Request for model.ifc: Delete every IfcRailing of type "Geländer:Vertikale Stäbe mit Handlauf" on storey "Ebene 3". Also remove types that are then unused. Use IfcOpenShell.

First a look at what the model holds.

```python
import ifcopenshell
import ifcopenshell.util.element

model = ifcopenshell.open("model.ifc")
print(model.schema)
storey = next(s for s in model.by_type("IfcBuildingStorey") if s.Name == "Ebene 3")
railings = [e for e in ifcopenshell.util.element.get_decomposition(storey) if e.is_a("IfcRailing")]
seen = {}
for e in railings:
    element_type = ifcopenshell.util.element.get_type(e)
    name = element_type.Name if element_type not in (None, e) else None
    seen[name] = seen.get(name, 0) + 1
for name, count in sorted(seen.items(), key=str):
    print(count, "x", name)
```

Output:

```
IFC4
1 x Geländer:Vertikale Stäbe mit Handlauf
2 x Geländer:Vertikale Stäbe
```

```python
import ifcopenshell
import ifcopenshell.api.root
import ifcopenshell.util.element

model = ifcopenshell.open("model.ifc")

storey = next(s for s in model.by_type("IfcBuildingStorey") if s.Name == "Ebene 3")
railings = [e for e in ifcopenshell.util.element.get_decomposition(storey) if e.is_a("IfcRailing")]
targets = [e for e in railings if (t := ifcopenshell.util.element.get_type(e)) not in (None, e) and t.Name == "Geländer:Vertikale Stäbe mit Handlauf"]
types = {ifcopenshell.util.element.get_type(e) for e in targets} - {None, *targets}

for e in targets:
    ifcopenshell.api.root.remove_product(model, product=e)
print(len(targets), "removed")

unused = [t for t in types if not ifcopenshell.util.element.get_types(t)]
for t in unused:
    ifcopenshell.api.root.remove_product(model, product=t)
print(len(unused), "unused types removed")

model.write("model_edited.ifc")
```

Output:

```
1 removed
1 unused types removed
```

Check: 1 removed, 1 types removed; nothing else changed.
